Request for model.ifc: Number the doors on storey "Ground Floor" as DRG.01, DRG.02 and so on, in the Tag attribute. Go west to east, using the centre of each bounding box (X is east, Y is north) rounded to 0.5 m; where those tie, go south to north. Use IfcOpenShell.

First a look at what the model holds.

```python
import ifcopenshell
import ifcopenshell.util.element
import ifcopenshell.util.placement

model = ifcopenshell.open("model.ifc")
print(model.schema)
storey = next(s for s in model.by_type("IfcBuildingStorey") if s.Name == "Ground Floor")
doors = [e for e in ifcopenshell.util.element.get_decomposition(storey) if e.is_a("IfcDoor")]
for e in sorted(doors, key=lambda e: e.id()):
    origin = ifcopenshell.util.placement.get_local_placement(e.ObjectPlacement)[:3, 3]
    print(e.id(), e.Tag, e.Name, origin.round(2) + 0.0, sep=" | ")
```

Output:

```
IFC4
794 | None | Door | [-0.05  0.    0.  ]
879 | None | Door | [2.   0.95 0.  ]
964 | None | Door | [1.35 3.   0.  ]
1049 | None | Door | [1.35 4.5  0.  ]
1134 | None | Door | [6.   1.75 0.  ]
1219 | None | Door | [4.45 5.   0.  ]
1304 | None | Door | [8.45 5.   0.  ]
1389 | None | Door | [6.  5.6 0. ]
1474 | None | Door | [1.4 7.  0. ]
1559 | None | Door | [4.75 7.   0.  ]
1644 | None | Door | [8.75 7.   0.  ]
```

```python
import ifcopenshell
import ifcopenshell.geom
import ifcopenshell.util.element
import ifcopenshell.util.shape

model = ifcopenshell.open("model.ifc")
settings = ifcopenshell.geom.settings()
settings.set("use-world-coords", True)


def centre(element):
    shape = ifcopenshell.geom.create_shape(settings, element)
    return ifcopenshell.util.shape.get_bbox_centroid(shape.geometry)


storey = next(s for s in model.by_type("IfcBuildingStorey") if s.Name == "Ground Floor")
doors = [e for e in ifcopenshell.util.element.get_decomposition(storey) if e.is_a("IfcDoor")]

# Insertion points can sit at a corner or the storey origin, so sort by the geometry (in metres).
centres = {e: centre(e) for e in doors}
doors.sort(key=lambda e: (round(centres[e][0] / 0.5), centres[e][1]))

for i, e in enumerate(doors, start=1):
    number = f"DRG.{i:02d}"
    e.Tag = number
    print(e.id(), number)

model.write("model_v2.ifc")
```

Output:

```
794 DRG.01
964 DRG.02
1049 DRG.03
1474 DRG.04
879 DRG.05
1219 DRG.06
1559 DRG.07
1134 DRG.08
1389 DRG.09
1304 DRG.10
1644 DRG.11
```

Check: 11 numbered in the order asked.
